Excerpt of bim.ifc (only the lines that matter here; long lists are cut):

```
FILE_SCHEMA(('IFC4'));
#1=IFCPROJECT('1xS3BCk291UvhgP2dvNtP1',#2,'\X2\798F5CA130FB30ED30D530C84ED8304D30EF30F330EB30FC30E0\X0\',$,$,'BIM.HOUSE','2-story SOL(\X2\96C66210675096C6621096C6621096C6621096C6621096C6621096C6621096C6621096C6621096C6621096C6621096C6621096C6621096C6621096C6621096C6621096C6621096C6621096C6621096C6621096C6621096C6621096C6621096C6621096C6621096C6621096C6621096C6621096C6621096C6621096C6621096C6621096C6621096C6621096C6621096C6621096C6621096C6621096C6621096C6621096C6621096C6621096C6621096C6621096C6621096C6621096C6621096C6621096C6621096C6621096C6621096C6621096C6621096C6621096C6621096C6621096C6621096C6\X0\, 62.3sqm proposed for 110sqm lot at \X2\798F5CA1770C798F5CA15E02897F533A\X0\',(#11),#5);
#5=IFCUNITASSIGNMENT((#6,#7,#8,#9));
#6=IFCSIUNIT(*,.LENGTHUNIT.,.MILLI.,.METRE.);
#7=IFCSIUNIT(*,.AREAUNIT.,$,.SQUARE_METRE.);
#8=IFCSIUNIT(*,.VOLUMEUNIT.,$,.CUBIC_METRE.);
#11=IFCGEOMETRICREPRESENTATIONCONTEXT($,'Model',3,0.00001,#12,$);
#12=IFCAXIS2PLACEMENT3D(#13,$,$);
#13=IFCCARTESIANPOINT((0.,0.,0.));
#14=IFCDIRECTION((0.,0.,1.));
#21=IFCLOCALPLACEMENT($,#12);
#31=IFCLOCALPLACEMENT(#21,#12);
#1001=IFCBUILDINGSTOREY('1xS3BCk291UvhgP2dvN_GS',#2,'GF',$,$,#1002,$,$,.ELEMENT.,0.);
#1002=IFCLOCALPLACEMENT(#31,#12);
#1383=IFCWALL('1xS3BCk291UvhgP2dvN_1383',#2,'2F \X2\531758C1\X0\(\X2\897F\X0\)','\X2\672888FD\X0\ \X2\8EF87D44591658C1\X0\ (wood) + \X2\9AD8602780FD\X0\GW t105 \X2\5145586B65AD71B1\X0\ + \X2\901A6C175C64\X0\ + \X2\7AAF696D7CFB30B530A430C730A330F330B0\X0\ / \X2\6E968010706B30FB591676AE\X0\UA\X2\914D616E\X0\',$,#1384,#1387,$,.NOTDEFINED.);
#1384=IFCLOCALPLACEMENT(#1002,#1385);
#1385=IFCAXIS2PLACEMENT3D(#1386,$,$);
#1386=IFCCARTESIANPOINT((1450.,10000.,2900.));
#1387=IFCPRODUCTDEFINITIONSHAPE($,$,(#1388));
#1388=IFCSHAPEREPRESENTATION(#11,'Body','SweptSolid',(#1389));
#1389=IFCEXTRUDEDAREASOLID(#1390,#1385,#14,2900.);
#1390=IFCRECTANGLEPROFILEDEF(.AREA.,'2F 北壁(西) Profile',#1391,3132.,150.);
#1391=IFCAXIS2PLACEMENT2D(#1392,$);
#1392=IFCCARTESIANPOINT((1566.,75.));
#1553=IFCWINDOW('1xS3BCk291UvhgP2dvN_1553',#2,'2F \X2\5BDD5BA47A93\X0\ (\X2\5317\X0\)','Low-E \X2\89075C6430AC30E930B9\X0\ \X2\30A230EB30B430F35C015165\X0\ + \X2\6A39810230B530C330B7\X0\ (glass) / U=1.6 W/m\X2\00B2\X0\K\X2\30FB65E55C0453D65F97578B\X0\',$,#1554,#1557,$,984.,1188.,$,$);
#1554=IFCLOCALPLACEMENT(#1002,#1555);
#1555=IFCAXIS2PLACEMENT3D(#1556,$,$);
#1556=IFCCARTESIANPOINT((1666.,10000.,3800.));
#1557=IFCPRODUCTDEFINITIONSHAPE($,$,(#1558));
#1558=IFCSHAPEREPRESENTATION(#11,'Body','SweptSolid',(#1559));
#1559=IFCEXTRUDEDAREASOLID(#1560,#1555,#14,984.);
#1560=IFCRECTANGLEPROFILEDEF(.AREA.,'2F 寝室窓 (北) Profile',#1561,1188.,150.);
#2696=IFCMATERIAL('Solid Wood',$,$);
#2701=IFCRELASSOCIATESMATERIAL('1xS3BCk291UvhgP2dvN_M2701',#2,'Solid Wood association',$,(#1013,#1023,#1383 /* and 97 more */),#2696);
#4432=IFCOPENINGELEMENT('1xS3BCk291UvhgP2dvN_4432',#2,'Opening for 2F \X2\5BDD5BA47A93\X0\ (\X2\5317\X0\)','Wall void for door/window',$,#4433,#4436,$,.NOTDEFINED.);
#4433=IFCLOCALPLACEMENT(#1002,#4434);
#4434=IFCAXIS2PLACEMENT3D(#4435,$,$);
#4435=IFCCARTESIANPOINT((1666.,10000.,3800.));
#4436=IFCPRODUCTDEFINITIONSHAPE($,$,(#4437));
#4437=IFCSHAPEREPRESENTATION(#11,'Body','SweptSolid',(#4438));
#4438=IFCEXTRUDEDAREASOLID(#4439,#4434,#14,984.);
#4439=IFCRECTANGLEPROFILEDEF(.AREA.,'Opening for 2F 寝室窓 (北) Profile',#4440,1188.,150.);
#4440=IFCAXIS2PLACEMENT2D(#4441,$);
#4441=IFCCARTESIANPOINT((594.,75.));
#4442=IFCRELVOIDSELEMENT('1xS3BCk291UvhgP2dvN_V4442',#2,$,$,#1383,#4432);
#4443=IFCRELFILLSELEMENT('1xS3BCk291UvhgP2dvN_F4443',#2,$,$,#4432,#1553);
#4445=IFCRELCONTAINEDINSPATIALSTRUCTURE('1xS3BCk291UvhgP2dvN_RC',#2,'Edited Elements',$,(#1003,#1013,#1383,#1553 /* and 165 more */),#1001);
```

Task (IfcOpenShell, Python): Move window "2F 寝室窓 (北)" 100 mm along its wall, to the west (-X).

```python
import ifcopenshell
import ifcopenshell.api.geometry
import ifcopenshell.util.placement

model = ifcopenshell.open("bim.ifc")

window = model.by_guid("1xS3BCk291UvhgP2dvN_1553")
opening = window.FillsVoids[0].RelatingOpeningElement
wall = opening.VoidsElements[0].RelatingBuildingElement

wall_matrix = ifcopenshell.util.placement.get_local_placement(wall.ObjectPlacement)
shift = wall_matrix[:3, 0] * -100.0
before = ifcopenshell.util.placement.get_local_placement(window.ObjectPlacement)[:3, 3].copy()

# The window is not placed relative to its opening, so move both.
for product in (opening, window):
    matrix = ifcopenshell.util.placement.get_local_placement(product.ObjectPlacement)
    matrix[:3, 3] += shift
    ifcopenshell.api.geometry.edit_object_placement(model, product=product, matrix=matrix, is_si=False)

after = ifcopenshell.util.placement.get_local_placement(window.ObjectPlacement)[:3, 3]
print("window moved by", (after - before).round(3) + 0.0)

model.write("bim-out.ifc")
```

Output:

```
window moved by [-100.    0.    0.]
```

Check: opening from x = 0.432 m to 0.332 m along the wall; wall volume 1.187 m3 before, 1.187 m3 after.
